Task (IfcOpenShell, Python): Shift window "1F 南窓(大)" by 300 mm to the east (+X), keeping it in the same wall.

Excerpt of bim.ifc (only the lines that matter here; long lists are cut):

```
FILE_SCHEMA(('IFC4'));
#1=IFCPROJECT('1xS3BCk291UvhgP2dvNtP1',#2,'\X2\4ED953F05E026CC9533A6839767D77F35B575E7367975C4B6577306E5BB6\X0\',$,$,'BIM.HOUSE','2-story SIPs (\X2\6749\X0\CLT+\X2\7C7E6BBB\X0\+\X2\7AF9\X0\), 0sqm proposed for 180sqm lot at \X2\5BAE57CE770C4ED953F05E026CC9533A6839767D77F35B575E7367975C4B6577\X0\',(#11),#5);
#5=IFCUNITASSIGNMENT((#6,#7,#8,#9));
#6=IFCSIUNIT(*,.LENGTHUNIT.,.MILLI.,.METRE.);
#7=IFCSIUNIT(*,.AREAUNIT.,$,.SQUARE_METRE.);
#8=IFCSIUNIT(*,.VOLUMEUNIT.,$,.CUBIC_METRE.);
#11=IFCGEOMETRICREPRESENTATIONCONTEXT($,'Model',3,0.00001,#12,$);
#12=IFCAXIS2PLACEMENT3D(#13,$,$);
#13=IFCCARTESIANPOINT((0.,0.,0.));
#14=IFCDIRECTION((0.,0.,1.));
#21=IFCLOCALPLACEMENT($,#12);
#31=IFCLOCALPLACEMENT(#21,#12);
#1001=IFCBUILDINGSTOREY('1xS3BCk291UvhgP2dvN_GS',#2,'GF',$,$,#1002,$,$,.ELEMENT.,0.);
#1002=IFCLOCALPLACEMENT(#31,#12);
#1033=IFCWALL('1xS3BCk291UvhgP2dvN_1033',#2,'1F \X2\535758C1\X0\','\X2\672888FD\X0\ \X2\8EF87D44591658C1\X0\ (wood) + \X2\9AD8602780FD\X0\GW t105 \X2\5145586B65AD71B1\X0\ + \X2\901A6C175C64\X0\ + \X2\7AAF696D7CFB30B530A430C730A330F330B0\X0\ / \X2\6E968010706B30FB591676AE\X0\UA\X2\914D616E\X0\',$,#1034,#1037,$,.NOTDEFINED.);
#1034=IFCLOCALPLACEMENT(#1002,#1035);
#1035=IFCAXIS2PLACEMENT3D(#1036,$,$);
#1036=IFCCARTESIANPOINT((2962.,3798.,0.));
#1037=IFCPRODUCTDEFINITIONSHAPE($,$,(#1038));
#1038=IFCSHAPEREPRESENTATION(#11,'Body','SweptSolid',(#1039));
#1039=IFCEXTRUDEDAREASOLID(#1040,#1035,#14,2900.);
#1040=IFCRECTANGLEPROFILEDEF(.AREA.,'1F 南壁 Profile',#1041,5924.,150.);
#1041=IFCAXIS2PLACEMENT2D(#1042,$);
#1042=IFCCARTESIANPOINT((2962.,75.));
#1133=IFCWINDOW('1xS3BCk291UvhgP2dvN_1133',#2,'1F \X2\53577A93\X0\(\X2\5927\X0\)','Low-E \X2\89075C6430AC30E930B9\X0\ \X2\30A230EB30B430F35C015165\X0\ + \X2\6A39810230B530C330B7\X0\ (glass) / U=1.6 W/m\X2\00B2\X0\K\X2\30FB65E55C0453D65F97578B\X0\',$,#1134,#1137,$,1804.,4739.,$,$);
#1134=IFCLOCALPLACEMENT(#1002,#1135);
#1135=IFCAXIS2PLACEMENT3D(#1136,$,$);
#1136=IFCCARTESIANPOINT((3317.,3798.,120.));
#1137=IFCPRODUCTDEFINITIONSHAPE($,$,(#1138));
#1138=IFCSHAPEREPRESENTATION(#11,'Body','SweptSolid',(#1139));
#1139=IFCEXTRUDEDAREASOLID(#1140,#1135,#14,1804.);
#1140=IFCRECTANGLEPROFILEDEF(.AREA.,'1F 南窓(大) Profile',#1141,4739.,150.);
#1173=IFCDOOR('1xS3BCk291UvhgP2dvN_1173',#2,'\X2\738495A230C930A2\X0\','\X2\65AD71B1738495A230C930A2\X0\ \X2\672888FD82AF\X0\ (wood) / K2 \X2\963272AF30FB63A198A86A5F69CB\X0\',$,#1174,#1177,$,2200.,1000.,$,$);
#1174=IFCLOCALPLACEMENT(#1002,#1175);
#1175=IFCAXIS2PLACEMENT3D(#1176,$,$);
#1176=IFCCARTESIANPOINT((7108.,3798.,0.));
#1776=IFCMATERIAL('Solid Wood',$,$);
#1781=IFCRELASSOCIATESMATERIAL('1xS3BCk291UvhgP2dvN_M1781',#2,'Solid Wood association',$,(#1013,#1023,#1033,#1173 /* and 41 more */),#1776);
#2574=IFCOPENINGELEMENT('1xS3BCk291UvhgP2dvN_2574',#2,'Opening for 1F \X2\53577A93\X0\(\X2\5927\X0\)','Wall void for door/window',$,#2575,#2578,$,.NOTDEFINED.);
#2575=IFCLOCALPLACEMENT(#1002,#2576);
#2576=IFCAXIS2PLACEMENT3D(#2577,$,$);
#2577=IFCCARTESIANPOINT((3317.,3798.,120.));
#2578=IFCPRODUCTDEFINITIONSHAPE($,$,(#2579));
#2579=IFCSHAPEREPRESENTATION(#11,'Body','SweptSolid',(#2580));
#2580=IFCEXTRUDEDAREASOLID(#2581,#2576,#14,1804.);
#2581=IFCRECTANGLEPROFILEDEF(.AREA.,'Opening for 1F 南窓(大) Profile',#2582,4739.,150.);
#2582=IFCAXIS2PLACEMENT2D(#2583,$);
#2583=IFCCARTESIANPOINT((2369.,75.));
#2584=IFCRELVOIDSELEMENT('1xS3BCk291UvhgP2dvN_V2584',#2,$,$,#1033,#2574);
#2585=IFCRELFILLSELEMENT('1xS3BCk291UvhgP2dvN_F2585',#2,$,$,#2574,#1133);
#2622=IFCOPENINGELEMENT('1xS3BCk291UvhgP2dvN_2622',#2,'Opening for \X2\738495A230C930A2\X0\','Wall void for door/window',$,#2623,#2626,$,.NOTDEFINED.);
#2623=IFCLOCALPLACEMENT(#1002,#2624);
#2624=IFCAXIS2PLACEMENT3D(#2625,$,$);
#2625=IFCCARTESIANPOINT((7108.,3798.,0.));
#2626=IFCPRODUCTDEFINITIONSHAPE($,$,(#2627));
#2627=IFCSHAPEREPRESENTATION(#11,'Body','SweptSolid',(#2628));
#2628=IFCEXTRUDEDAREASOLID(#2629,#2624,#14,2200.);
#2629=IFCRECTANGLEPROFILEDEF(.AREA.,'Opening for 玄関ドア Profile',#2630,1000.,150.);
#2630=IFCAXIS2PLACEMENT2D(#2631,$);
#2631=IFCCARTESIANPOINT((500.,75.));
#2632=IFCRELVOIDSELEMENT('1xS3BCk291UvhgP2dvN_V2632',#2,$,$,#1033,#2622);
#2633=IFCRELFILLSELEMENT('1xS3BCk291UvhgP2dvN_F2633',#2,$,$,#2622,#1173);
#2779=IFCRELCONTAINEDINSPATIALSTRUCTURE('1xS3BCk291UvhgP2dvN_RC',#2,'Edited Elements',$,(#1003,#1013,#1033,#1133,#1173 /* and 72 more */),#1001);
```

```python
import ifcopenshell
import ifcopenshell.api.geometry
import ifcopenshell.util.placement
import ifcopenshell.util.unit

model = ifcopenshell.open("bim.ifc")
unit_scale = ifcopenshell.util.unit.calculate_unit_scale(model)

window = model.by_guid("1xS3BCk291UvhgP2dvN_1133")
opening = window.FillsVoids[0].RelatingOpeningElement
wall = opening.VoidsElements[0].RelatingBuildingElement

wall_matrix = ifcopenshell.util.placement.get_local_placement(wall.ObjectPlacement)
shift = wall_matrix[:3, 0] * 0.3 / unit_scale
before = ifcopenshell.util.placement.get_local_placement(window.ObjectPlacement)[:3, 3].copy()

# The window is not placed relative to its opening, so move both.
for product in (opening, window):
    matrix = ifcopenshell.util.placement.get_local_placement(product.ObjectPlacement)
    matrix[:3, 3] += shift
    ifcopenshell.api.geometry.edit_object_placement(model, product=product, matrix=matrix, is_si=False)

after = ifcopenshell.util.placement.get_local_placement(window.ObjectPlacement)[:3, 3]
print("window moved by", (after - before).round(3) + 0.0)

model.write("bim_rev.ifc")
```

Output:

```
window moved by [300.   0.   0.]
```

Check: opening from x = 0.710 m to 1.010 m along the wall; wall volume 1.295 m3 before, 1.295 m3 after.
